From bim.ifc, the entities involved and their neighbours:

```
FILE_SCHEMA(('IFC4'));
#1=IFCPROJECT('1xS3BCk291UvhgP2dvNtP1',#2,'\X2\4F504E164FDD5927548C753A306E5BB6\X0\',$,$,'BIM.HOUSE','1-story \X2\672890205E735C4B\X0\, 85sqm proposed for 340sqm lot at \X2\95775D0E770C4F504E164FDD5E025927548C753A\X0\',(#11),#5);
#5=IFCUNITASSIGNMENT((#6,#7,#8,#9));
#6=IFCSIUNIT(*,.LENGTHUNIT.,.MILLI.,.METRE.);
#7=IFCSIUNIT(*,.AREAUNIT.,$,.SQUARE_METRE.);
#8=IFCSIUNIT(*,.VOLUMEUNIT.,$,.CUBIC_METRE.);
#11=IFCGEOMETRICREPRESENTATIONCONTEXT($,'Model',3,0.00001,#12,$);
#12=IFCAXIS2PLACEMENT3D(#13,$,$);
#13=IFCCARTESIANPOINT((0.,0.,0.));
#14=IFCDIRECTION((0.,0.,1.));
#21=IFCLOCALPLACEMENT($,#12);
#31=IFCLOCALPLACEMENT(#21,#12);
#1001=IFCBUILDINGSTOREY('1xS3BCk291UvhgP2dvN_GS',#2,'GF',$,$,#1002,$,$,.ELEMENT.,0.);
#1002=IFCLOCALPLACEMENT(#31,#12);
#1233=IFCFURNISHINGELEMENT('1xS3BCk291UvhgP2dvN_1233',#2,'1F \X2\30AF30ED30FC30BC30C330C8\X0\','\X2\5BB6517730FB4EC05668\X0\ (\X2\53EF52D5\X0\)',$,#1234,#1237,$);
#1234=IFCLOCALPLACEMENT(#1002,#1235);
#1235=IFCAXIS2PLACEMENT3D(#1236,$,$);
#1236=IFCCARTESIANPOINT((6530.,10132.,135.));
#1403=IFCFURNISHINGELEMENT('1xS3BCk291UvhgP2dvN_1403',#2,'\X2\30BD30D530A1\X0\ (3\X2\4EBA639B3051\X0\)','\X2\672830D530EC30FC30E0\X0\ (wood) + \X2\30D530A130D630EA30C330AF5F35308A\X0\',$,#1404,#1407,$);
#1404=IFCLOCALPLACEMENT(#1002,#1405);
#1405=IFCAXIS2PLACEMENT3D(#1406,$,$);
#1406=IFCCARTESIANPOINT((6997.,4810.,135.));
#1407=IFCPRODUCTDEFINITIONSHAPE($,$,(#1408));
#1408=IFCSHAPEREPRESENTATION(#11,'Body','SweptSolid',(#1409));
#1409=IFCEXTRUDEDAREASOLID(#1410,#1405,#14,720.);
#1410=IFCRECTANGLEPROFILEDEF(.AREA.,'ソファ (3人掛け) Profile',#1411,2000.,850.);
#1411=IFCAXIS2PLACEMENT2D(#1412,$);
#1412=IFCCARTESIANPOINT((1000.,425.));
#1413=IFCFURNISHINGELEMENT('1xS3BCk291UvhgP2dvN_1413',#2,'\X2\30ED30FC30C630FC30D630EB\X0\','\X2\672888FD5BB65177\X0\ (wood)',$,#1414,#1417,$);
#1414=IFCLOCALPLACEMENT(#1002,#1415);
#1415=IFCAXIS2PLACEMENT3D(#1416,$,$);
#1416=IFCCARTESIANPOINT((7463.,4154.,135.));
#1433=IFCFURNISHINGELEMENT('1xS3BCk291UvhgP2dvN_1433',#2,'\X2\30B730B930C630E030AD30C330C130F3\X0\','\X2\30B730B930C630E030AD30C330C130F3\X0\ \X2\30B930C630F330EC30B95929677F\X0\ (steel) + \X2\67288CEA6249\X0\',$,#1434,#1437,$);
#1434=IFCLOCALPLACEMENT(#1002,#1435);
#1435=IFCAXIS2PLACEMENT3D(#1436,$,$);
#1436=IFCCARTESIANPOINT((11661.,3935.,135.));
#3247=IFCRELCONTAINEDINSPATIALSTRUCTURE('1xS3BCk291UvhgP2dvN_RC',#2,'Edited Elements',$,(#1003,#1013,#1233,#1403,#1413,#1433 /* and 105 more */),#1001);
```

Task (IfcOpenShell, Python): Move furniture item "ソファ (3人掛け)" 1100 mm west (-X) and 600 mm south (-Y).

```python
import ifcopenshell
import ifcopenshell.api.geometry
import ifcopenshell.util.placement
import ifcopenshell.util.unit

model = ifcopenshell.open("bim.ifc")
unit_scale = ifcopenshell.util.unit.calculate_unit_scale(model)

item = model.by_guid("1xS3BCk291UvhgP2dvN_1403")
matrix = ifcopenshell.util.placement.get_local_placement(item.ObjectPlacement)
matrix[0, 3] -= 1.1 / unit_scale
matrix[1, 3] -= 0.6 / unit_scale
ifcopenshell.api.geometry.edit_object_placement(model, product=item, matrix=matrix, is_si=False)

print(ifcopenshell.util.placement.get_local_placement(item.ObjectPlacement).round(3) + 0.0)

model.write("bim_v2.ifc")
```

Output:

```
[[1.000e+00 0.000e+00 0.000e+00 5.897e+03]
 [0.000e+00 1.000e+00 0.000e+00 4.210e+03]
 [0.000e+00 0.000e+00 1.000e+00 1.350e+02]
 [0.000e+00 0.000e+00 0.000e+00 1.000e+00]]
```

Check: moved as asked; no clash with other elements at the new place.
